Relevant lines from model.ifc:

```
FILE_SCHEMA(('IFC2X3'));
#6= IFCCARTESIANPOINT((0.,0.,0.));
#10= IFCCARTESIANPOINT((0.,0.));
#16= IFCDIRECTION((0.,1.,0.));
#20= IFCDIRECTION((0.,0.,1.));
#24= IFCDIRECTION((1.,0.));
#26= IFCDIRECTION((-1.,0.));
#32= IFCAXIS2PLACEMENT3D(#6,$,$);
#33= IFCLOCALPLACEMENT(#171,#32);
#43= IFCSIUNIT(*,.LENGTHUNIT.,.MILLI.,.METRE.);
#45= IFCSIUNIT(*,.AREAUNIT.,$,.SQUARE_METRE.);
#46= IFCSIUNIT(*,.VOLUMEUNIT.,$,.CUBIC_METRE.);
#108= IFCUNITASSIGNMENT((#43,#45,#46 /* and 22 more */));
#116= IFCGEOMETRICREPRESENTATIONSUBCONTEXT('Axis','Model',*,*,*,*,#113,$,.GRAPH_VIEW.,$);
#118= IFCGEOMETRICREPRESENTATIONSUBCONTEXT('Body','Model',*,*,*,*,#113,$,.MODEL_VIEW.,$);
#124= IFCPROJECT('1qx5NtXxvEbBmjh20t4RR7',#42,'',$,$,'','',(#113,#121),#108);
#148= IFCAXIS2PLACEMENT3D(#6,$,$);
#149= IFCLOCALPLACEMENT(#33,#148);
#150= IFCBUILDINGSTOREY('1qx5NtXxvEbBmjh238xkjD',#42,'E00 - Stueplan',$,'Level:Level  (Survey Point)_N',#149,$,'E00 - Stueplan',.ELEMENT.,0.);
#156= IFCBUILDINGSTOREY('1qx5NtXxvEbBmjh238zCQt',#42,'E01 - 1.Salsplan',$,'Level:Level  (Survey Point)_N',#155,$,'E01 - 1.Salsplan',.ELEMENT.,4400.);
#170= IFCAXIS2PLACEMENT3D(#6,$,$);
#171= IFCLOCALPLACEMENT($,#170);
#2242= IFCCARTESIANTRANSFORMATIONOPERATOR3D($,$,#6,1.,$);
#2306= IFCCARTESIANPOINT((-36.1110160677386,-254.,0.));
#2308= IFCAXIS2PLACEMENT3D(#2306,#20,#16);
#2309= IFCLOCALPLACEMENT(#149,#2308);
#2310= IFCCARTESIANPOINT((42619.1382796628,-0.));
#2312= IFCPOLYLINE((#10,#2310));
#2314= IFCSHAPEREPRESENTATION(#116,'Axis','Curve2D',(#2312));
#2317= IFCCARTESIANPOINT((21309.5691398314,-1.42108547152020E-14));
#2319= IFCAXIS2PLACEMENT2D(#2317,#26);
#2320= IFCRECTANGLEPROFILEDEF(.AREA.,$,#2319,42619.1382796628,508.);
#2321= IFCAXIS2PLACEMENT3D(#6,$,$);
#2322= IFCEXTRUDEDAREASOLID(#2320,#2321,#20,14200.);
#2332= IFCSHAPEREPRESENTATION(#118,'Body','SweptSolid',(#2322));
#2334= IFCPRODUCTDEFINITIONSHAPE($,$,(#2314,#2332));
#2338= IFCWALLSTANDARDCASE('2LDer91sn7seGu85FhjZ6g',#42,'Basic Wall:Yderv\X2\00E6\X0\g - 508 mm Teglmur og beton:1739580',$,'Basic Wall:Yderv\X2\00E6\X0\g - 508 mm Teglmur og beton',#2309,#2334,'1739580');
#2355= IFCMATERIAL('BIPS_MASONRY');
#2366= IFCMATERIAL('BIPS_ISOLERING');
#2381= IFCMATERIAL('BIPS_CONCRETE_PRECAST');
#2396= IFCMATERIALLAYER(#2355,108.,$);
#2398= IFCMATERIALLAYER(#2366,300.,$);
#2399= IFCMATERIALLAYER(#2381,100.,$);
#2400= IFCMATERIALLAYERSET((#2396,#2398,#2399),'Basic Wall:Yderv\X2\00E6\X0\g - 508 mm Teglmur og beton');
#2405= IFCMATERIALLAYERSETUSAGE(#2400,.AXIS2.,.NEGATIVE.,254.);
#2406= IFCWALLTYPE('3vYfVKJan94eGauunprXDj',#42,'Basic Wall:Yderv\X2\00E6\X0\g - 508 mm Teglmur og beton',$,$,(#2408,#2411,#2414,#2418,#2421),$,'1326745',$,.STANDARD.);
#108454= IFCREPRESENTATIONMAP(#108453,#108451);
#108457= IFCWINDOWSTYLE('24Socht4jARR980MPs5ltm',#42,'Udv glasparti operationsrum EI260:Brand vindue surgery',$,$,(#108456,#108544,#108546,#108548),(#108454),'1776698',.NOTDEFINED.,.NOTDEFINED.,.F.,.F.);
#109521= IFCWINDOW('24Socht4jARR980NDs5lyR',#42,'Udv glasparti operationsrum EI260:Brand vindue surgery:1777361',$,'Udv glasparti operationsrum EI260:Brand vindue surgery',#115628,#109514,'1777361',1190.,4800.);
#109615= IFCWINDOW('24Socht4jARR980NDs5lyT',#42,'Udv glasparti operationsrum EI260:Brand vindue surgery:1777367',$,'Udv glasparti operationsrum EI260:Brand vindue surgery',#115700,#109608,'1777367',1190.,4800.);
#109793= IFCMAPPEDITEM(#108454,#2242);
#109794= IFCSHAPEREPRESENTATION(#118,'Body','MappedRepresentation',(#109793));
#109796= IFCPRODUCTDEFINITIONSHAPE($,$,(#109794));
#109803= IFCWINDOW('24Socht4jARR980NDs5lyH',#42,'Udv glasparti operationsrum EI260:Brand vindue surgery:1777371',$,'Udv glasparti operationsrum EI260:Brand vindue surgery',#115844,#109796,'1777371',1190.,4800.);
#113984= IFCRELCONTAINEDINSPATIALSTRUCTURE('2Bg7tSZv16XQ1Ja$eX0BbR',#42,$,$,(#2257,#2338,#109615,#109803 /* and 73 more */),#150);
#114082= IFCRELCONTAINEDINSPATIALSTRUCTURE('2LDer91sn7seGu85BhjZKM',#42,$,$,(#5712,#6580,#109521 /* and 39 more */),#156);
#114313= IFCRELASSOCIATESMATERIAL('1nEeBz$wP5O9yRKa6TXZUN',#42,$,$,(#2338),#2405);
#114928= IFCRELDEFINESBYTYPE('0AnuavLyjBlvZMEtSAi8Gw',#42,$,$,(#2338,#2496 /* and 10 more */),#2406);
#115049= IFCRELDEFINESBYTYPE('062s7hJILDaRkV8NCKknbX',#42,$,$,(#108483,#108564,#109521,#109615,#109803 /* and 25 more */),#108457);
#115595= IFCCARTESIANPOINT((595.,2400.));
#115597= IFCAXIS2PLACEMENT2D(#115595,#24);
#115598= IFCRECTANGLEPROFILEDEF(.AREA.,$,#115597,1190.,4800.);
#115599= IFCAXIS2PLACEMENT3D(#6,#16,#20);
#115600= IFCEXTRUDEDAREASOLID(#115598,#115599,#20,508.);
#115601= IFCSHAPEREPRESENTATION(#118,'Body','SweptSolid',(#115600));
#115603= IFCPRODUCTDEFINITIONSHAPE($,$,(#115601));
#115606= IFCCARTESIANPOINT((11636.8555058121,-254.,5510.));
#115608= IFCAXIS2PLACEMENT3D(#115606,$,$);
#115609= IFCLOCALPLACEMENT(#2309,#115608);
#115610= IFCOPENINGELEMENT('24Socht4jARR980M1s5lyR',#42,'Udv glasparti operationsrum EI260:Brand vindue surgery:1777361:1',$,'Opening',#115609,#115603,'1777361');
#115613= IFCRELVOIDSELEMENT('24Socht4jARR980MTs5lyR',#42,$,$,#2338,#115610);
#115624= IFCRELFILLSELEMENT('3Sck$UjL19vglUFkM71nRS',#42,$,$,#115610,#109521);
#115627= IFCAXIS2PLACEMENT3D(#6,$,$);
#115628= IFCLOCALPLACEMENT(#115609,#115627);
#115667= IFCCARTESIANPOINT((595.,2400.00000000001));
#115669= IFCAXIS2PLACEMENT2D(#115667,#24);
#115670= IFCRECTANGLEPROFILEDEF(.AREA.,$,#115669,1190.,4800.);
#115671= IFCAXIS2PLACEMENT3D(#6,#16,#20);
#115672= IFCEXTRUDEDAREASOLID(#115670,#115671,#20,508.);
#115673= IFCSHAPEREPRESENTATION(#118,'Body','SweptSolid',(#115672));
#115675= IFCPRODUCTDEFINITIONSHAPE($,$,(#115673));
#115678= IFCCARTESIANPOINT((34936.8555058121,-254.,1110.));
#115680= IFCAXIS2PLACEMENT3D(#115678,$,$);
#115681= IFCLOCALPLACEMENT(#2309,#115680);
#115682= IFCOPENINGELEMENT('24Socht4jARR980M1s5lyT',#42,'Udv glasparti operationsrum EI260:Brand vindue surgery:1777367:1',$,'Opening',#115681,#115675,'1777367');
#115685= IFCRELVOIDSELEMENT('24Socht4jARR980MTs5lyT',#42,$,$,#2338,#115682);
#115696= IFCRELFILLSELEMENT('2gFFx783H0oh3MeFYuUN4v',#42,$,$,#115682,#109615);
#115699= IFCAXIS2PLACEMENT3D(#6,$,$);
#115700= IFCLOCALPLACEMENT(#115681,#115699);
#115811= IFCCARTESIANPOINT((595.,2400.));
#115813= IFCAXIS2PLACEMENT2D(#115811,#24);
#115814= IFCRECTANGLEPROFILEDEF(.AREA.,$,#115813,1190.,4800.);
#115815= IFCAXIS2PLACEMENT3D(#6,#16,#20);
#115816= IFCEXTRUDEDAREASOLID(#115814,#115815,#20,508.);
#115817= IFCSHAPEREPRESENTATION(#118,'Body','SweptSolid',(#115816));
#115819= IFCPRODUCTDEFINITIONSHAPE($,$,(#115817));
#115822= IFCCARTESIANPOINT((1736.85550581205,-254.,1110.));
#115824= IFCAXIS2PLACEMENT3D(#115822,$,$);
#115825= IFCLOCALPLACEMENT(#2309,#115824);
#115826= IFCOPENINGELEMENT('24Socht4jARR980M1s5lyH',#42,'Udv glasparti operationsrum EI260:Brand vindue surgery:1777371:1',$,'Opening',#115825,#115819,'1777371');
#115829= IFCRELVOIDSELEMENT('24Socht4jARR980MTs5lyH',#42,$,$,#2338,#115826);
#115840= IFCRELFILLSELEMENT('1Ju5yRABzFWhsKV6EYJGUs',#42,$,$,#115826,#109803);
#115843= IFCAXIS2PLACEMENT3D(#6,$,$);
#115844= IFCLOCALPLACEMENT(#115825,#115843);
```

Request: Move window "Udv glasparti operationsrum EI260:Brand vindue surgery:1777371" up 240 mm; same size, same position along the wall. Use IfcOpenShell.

```python
import numpy as np
import ifcopenshell
import ifcopenshell.api.geometry
import ifcopenshell.util.placement
import ifcopenshell.util.unit

model = ifcopenshell.open("model.ifc")
unit_scale = ifcopenshell.util.unit.calculate_unit_scale(model)

window = model.by_guid("24Socht4jARR980NDs5lyH")
opening = window.FillsVoids[0].RelatingOpeningElement
dz = 0.24 / unit_scale

shift = np.array([0.0, 0.0, dz])
# The window is placed relative to its opening, so it follows when the opening moves.
matrix = ifcopenshell.util.placement.get_local_placement(opening.ObjectPlacement)
matrix[:3, 3] += shift
ifcopenshell.api.geometry.edit_object_placement(
    model, product=opening, matrix=matrix, is_si=False, should_transform_children=True
)

print(f"moved by {dz * unit_scale:+.3f} m")

model.write("model-out.ifc")
```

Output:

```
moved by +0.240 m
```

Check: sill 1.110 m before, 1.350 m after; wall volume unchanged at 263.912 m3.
